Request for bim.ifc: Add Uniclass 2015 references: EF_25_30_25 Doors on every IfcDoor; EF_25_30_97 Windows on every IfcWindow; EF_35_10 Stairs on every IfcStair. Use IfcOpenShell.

First a look at what the model holds.

```python
import ifcopenshell

model = ifcopenshell.open("bim.ifc")
print(model.schema)
print("classifications:", [c.Name for c in model.by_type("IfcClassification")])
for ifc_class in ("IfcDoor", "IfcRoof", "IfcStair", "IfcWall", "IfcWindow"):
    print(ifc_class, len(model.by_type(ifc_class)))
```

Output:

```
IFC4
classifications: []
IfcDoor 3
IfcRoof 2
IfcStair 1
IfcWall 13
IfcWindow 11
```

```python
import ifcopenshell
import ifcopenshell.api.classification

model = ifcopenshell.open("bim.ifc")

system = ifcopenshell.api.classification.add_classification(model, classification="Uniclass 2015")

codes = {
    "IfcDoor": ("EF_25_30_25", "Doors"),
    "IfcWindow": ("EF_25_30_97", "Windows"),
    "IfcStair": ("EF_35_10", "Stairs"),
}
for ifc_class, (code, name) in codes.items():
    products = model.by_type(ifc_class)
    ifcopenshell.api.classification.add_reference(
        model, products=products, classification=system, identification=code, name=name
    )
    print(code, len(products))

model.write("bim-out.ifc")
```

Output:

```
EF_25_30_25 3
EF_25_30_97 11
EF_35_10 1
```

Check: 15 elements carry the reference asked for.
